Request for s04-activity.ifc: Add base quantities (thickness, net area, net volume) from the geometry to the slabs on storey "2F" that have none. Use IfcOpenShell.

First a look at what the model holds.

```python
import ifcopenshell
import ifcopenshell.util.element
import ifcopenshell.util.unit

model = ifcopenshell.open("s04-activity.ifc")
print(model.schema)
for unit_type in ("LENGTHUNIT", "AREAUNIT", "VOLUMEUNIT"):
    print(unit_type, ifcopenshell.util.unit.calculate_unit_scale(model, unit_type))
storey = next(s for s in model.by_type("IfcBuildingStorey") if s.Name == "2F")
slabs = [e for e in ifcopenshell.util.element.get_decomposition(storey) if e.is_a("IfcSlab")]
for e in sorted(slabs, key=lambda e: e.id()):
    print(e.id(), e.is_a(), e.Name, list(ifcopenshell.util.element.get_psets(e, qtos_only=True)), sep=" | ")
```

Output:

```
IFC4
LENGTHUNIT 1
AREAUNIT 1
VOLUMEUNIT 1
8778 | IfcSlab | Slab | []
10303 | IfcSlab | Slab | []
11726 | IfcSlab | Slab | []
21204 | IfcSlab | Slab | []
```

```python
import ifcopenshell
import ifcopenshell.api.pset
import ifcopenshell.geom
import ifcopenshell.util.element
import ifcopenshell.util.shape
import ifcopenshell.util.unit

model = ifcopenshell.open("s04-activity.ifc")
unit_scale = ifcopenshell.util.unit.calculate_unit_scale(model)
area_scale = ifcopenshell.util.unit.calculate_unit_scale(model, "AREAUNIT")
volume_scale = ifcopenshell.util.unit.calculate_unit_scale(model, "VOLUMEUNIT")
settings = ifcopenshell.geom.settings()

storey = next(s for s in model.by_type("IfcBuildingStorey") if s.Name == "2F")
slabs = [e for e in ifcopenshell.util.element.get_decomposition(storey) if e.is_a("IfcSlab")]

for e in sorted(slabs, key=lambda e: e.id()):
    if ifcopenshell.util.element.get_psets(e, qtos_only=True, should_inherit=False):
        continue
    # Geometry comes back in metres, in the element's own axes.
    shape = ifcopenshell.geom.create_shape(settings, e)
    values = {
        "Width": ifcopenshell.util.shape.get_z(shape.geometry) / unit_scale,
        "NetArea": ifcopenshell.util.shape.get_footprint_area(shape.geometry) / area_scale,
        "NetVolume": ifcopenshell.util.shape.get_volume(shape.geometry) / volume_scale,
    }
    qto = ifcopenshell.api.pset.add_qto(model, product=e, name="Qto_SlabBaseQuantities")
    ifcopenshell.api.pset.edit_qto(model, qto=qto, properties=values)
    print(e.id(), {k: round(v, 3) for k, v in values.items()})

model.write("s04-activity_updated.ifc")
```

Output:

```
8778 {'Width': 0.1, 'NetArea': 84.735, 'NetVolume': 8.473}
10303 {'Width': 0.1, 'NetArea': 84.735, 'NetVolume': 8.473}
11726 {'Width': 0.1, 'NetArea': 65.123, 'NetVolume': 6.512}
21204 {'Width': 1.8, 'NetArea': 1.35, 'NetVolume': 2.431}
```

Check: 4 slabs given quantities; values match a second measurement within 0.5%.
